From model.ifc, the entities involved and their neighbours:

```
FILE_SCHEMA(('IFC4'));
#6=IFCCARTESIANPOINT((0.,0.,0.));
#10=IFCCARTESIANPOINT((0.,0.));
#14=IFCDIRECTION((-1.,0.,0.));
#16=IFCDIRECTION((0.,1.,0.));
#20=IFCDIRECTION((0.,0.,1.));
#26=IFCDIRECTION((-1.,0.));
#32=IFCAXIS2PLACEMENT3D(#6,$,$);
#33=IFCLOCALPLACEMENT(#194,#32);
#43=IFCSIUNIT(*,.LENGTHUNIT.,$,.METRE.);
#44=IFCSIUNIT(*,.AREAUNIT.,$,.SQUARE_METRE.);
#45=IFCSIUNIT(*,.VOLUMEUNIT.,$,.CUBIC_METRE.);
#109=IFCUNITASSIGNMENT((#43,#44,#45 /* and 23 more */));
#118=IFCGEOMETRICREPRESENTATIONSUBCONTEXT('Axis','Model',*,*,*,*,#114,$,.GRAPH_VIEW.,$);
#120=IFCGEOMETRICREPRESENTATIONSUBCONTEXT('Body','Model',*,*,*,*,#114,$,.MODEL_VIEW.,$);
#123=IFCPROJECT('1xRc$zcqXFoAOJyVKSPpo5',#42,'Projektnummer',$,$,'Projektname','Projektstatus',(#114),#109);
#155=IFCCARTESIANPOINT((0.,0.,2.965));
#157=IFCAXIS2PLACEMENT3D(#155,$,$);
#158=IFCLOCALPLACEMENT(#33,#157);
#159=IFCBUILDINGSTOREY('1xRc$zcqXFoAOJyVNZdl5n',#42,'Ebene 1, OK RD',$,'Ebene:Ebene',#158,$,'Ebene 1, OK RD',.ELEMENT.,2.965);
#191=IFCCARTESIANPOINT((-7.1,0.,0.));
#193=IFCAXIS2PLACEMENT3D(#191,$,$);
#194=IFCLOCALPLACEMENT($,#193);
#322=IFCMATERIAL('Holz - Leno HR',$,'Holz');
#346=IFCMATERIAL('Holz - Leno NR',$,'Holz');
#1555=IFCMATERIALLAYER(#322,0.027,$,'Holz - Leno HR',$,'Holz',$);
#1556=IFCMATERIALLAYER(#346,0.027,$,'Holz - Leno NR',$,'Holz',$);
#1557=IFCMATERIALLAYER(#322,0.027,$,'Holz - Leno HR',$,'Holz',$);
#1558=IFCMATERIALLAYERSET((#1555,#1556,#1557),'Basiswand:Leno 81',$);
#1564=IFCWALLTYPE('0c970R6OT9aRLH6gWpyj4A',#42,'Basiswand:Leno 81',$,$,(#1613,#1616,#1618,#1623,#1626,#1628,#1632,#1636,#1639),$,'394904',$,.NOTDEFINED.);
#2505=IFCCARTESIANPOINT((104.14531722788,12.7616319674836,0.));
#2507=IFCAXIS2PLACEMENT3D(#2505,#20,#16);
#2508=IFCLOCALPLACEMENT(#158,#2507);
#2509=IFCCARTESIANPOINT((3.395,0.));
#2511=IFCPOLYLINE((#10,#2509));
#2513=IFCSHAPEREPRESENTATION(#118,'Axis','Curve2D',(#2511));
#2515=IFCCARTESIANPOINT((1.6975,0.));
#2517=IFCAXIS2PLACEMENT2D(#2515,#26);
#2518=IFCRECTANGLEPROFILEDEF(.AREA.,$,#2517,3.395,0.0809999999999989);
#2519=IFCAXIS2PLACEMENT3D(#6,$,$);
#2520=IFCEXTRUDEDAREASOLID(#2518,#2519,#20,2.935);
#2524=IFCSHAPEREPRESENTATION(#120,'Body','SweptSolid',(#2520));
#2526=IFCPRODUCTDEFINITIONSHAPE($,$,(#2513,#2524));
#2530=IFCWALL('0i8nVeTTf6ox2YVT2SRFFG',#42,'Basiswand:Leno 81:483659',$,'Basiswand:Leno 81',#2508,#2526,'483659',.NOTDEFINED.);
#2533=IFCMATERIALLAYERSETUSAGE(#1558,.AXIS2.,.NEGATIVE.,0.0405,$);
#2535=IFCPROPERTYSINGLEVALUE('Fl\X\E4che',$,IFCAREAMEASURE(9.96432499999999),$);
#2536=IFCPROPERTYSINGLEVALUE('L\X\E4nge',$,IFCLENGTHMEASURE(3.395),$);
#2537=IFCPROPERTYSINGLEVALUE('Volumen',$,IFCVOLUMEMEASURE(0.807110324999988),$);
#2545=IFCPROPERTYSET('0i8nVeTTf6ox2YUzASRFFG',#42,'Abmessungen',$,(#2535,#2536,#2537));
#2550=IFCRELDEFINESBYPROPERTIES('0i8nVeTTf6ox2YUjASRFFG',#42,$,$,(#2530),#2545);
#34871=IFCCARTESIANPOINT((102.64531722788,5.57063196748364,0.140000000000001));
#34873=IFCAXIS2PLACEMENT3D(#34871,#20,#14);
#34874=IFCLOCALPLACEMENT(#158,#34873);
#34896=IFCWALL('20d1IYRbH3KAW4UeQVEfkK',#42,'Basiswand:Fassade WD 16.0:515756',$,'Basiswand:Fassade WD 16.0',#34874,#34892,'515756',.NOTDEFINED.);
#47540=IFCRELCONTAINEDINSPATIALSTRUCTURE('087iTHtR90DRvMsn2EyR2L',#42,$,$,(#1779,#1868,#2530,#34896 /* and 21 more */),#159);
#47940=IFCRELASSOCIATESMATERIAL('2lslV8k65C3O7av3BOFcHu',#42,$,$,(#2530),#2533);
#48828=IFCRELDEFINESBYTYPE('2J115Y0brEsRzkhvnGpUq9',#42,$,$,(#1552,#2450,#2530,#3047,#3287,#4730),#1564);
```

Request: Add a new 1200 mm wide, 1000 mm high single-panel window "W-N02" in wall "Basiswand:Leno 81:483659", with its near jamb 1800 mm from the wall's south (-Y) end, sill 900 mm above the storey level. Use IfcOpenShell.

```python
import numpy as np
import ifcopenshell
import ifcopenshell.api.feature
import ifcopenshell.api.geometry
import ifcopenshell.api.pset
import ifcopenshell.api.root
import ifcopenshell.api.spatial
import ifcopenshell.geom
import ifcopenshell.util.element
import ifcopenshell.util.placement
import ifcopenshell.util.representation
import ifcopenshell.util.shape
import ifcopenshell.util.unit

model = ifcopenshell.open("model.ifc")
unit_scale = ifcopenshell.util.unit.calculate_unit_scale(model)
area_scale = ifcopenshell.util.unit.calculate_unit_scale(model, "AREAUNIT")
volume_scale = ifcopenshell.util.unit.calculate_unit_scale(model, "VOLUMEUNIT")
settings = ifcopenshell.geom.settings()


def volume(element):
    """Net volume in cubic metres, openings subtracted."""
    shape = ifcopenshell.geom.create_shape(settings, element)
    return ifcopenshell.util.shape.get_volume(shape.geometry)


wall = model.by_id(2530)
storey = ifcopenshell.util.element.get_container(wall, ifc_class="IfcBuildingStorey")
context = ifcopenshell.util.representation.get_context(model, "Model", "Body", "MODEL_VIEW")
before = volume(wall)

width, height, from_end, sill = 1.2, 1, 1.8, 0.9  # metres

# The wall runs along its own X axis, and the end named is its -X end.
wall_shape = ifcopenshell.geom.create_shape(settings, wall)
x, y, z = ifcopenshell.util.shape.get_vertices(wall_shape.geometry).T
start = x.min() + from_end
face, thickness = float(y.min()), float(y.max() - y.min())
wall_matrix = ifcopenshell.util.placement.get_local_placement(wall.ObjectPlacement)
level = ifcopenshell.util.placement.get_local_placement(storey.ObjectPlacement)[2, 3]


def in_wall(x, y):
    """Placement at x, y metres in the wall's axes, at sill height."""
    matrix = wall_matrix.copy()
    matrix[:, 3] = wall_matrix @ np.array([x / unit_scale, y / unit_scale, 0.0, 1.0])
    matrix[2, 3] = level + sill / unit_scale
    return matrix


# Opening: a box that overshoots both wall faces by 50 mm.
opening = ifcopenshell.api.root.create_entity(model, ifc_class="IfcOpeningElement", predefined_type="OPENING")
box = ifcopenshell.api.geometry.add_wall_representation(
    model, context=context, length=width, height=height, thickness=thickness + 0.1
)
ifcopenshell.api.geometry.assign_representation(model, product=opening, representation=box)
ifcopenshell.api.geometry.edit_object_placement(model, product=opening, matrix=in_wall(start, face - 0.05), is_si=False)
ifcopenshell.api.feature.add_feature(model, feature=opening, element=wall)

window = ifcopenshell.api.root.create_entity(model, ifc_class="IfcWindow", name="W-N02", predefined_type="WINDOW")
window.OverallWidth, window.OverallHeight = width / unit_scale, height / unit_scale
window.PartitioningType = "SINGLE_PANEL"
body = ifcopenshell.api.geometry.add_window_representation(
    model,
    context=context,
    overall_width=window.OverallWidth,
    overall_height=window.OverallHeight,
    partition_type="SINGLE_PANEL",
)
ifcopenshell.api.geometry.assign_representation(model, product=window, representation=body)
ifcopenshell.api.spatial.assign_container(model, products=[window], relating_structure=storey)
ifcopenshell.api.feature.add_filling(model, opening=opening, element=window)

# Centre the window in the wall's thickness.
ifcopenshell.api.geometry.edit_object_placement(model, product=window, matrix=in_wall(start, face), is_si=False)
window_shape = ifcopenshell.geom.create_shape(settings, window)
depth = ifcopenshell.util.shape.get_vertices(window_shape.geometry)[:, 1]
offset = face + thickness / 2 - (depth.min() + depth.max()) / 2
ifcopenshell.api.geometry.edit_object_placement(model, product=window, matrix=in_wall(start, offset), is_si=False)

after = volume(wall)

# Update the wall's stored quantities.
pset = model.by_id(ifcopenshell.util.element.get_pset(wall, "Abmessungen", should_inherit=False)["id"])
ifcopenshell.api.pset.edit_pset(model, pset=pset, properties={
    "Fläche": model.create_entity("IfcAreaMeasure", after / thickness / area_scale),
    "Volumen": model.create_entity("IfcVolumeMeasure", after / volume_scale),
})

print(f"wall volume {before:.3f} -> {after:.3f} m3")

model.write("model-out.ifc")
```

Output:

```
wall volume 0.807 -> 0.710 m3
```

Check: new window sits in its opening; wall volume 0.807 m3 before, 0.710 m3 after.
